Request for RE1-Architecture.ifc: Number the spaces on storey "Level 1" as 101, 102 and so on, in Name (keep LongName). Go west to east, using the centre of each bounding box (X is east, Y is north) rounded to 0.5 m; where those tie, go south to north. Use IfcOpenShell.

First a look at what the model holds.

```python
import ifcopenshell
import ifcopenshell.util.element
import ifcopenshell.util.placement

model = ifcopenshell.open("RE1-Architecture.ifc")
print(model.schema)
storey = next(s for s in model.by_type("IfcBuildingStorey") if s.Name == "Level 1")
spaces = [e for e in ifcopenshell.util.element.get_decomposition(storey) if e.is_a("IfcSpace")]
for e in sorted(spaces, key=lambda e: e.id()):
    origin = ifcopenshell.util.placement.get_local_placement(e.ObjectPlacement)[:3, 3]
    print(e.id(), e.Name, e.LongName, origin.round(2) + 0.0, sep=" | ")
```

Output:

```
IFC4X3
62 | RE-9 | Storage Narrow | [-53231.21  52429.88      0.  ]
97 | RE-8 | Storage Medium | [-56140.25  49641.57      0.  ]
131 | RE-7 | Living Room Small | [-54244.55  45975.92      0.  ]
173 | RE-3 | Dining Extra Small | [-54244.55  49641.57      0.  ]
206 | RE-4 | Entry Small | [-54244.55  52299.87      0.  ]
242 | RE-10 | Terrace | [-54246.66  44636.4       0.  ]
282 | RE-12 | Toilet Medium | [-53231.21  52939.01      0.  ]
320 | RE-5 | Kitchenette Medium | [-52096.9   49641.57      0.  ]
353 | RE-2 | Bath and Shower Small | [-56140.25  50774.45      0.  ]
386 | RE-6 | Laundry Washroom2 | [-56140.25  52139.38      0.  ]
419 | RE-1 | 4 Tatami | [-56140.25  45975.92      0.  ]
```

```python
import ifcopenshell
import ifcopenshell.geom
import ifcopenshell.util.element
import ifcopenshell.util.shape

model = ifcopenshell.open("RE1-Architecture.ifc")
settings = ifcopenshell.geom.settings()
settings.set("use-world-coords", True)


def centre(element):
    shape = ifcopenshell.geom.create_shape(settings, element)
    return ifcopenshell.util.shape.get_bbox_centroid(shape.geometry)


storey = next(s for s in model.by_type("IfcBuildingStorey") if s.Name == "Level 1")
spaces = [e for e in ifcopenshell.util.element.get_decomposition(storey) if e.is_a("IfcSpace")]

# Insertion points can sit at a corner or the storey origin, so sort by the geometry (in metres).
centres = {e: centre(e) for e in spaces}
spaces.sort(key=lambda e: (round(centres[e][0] / 0.5), centres[e][1]))

for i, e in enumerate(spaces, start=1):
    number = f"1{i:02d}"
    e.Name = number
    print(e.id(), number)

model.write("RE1-Architecture-out.ifc")
```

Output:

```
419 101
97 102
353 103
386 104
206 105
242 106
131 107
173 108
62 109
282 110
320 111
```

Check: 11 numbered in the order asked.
